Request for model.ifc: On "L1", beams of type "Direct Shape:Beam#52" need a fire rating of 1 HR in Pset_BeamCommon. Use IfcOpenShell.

First a look at what the model holds.

```python
import ifcopenshell
import ifcopenshell.util.element

model = ifcopenshell.open("model.ifc")
print(model.schema)
storey = next(s for s in model.by_type("IfcBuildingStorey") if s.Name == "L1")
beams = [e for e in ifcopenshell.util.element.get_decomposition(storey) if e.is_a("IfcBeam")]
seen = {}
for e in beams:
    element_type = ifcopenshell.util.element.get_type(e)
    key = (element_type.Name if element_type != e and element_type else None, ifcopenshell.util.element.get_pset(e, "Pset_BeamCommon", "FireRating"))
    seen[key] = seen.get(key, 0) + 1
for (name, value), count in sorted(seen.items(), key=str):
    print(count, "x", name, "|", value)
```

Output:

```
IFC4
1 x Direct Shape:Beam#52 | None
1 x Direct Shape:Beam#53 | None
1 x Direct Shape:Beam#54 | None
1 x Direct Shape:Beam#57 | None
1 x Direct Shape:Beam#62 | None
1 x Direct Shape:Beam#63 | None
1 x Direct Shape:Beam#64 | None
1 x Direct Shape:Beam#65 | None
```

```python
import ifcopenshell
import ifcopenshell.api.pset
import ifcopenshell.util.element

model = ifcopenshell.open("model.ifc")

storey = next(s for s in model.by_type("IfcBuildingStorey") if s.Name == "L1")
beams = [e for e in ifcopenshell.util.element.get_decomposition(storey) if e.is_a("IfcBeam")]

count = 0
for e in beams:
    element_type = ifcopenshell.util.element.get_type(e)
    if element_type in (None, e) or element_type.Name != "Direct Shape:Beam#52":
        continue
    # add_pset returns the element's existing set when there is one.
    pset = ifcopenshell.api.pset.add_pset(model, product=e, name="Pset_BeamCommon")
    ifcopenshell.api.pset.edit_pset(model, pset=pset, properties={"FireRating": "1 HR"})
    count += 1

print(count, "beams updated")

model.write("model_rev.ifc")
```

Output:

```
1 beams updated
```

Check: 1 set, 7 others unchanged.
